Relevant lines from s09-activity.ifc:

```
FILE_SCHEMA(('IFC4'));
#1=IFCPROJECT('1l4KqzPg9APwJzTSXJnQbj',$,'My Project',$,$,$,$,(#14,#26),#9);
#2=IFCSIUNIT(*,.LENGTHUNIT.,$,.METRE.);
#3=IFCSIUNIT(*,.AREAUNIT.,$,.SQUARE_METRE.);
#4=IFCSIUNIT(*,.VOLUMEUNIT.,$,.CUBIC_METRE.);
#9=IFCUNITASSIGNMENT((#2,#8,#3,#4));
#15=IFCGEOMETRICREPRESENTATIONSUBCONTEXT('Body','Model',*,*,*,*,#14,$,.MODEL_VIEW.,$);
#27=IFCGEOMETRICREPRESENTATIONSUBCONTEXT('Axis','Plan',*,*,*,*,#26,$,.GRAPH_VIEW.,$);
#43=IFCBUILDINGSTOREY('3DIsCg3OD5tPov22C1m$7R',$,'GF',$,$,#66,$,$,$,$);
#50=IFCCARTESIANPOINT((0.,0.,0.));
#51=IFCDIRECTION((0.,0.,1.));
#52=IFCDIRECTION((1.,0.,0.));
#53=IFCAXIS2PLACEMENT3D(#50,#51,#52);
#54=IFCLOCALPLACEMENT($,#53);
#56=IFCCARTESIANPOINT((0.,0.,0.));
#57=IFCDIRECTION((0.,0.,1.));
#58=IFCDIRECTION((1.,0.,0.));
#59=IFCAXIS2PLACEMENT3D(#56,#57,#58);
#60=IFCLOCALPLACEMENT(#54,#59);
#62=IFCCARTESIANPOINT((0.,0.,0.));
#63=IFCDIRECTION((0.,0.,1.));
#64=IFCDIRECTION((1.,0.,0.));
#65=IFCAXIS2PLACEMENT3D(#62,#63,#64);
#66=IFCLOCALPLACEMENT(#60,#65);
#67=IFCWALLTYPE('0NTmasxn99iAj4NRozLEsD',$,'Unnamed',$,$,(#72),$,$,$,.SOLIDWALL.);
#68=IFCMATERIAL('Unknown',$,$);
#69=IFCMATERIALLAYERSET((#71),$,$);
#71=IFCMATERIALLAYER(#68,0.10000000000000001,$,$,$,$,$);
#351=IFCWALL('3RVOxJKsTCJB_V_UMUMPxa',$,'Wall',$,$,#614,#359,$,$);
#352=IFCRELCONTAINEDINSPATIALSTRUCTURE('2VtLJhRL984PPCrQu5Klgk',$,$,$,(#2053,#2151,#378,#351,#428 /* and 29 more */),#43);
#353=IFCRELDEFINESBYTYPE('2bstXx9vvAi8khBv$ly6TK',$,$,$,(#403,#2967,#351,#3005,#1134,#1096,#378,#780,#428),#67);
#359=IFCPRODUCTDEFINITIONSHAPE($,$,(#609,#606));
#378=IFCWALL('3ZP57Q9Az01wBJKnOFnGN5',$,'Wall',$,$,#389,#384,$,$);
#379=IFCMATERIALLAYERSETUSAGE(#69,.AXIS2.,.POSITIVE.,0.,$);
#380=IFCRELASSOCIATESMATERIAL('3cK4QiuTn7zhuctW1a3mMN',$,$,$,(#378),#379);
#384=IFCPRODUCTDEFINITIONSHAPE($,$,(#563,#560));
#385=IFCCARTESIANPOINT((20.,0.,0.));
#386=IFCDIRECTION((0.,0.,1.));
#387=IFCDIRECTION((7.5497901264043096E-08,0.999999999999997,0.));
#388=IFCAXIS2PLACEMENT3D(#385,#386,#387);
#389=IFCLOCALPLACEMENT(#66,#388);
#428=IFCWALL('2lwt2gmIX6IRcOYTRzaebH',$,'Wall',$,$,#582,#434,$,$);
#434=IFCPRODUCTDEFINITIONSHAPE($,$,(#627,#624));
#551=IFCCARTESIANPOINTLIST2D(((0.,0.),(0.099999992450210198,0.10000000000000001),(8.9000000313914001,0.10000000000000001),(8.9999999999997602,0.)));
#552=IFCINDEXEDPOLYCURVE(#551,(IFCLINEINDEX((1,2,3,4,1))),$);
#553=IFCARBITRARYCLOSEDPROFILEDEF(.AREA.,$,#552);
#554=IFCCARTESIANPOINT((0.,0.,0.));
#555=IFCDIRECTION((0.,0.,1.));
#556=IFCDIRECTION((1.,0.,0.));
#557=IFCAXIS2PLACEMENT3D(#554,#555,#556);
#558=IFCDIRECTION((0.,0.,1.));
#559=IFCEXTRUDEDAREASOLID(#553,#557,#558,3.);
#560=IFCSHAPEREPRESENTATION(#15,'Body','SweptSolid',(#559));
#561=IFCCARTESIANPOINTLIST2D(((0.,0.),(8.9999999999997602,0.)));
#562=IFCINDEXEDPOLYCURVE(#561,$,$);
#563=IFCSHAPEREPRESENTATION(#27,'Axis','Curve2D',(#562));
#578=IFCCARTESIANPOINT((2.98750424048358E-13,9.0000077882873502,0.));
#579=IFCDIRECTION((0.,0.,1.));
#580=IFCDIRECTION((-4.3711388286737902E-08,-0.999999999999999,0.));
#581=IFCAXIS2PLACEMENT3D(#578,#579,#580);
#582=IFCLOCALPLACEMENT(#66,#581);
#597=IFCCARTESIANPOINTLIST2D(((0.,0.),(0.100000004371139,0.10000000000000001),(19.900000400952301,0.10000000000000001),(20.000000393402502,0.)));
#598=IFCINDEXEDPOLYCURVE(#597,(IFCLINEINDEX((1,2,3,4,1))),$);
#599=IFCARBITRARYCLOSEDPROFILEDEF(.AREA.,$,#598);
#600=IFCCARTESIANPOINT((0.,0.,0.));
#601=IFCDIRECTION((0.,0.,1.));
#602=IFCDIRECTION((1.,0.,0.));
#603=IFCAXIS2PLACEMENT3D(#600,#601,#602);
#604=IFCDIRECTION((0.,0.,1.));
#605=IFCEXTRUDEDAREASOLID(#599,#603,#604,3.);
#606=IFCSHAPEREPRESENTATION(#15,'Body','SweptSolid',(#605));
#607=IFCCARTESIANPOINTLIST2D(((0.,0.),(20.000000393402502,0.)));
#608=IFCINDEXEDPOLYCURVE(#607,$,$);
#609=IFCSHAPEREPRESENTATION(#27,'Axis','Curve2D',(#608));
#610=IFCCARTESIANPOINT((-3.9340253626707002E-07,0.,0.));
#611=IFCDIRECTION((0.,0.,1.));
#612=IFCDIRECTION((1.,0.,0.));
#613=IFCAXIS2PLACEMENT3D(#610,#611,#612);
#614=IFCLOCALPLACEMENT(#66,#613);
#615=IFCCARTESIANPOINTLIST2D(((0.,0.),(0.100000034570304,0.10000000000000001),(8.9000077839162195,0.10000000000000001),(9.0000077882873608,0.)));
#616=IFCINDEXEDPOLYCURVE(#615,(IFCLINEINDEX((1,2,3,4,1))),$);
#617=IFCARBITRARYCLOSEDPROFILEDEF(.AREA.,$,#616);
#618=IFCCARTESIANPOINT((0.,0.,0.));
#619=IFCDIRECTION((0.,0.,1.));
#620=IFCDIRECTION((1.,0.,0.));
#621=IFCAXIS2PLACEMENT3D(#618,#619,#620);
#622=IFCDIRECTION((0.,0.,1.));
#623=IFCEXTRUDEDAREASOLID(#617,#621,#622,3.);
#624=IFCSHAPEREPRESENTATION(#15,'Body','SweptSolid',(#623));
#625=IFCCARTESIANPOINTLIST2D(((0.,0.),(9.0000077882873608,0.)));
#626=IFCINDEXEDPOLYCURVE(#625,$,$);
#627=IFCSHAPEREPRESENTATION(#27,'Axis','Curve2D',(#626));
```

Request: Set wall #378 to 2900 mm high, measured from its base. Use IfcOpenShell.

```python
import ifcopenshell
import ifcopenshell.geom
import ifcopenshell.util.representation
import ifcopenshell.util.shape

model = ifcopenshell.open("s09-activity.ifc")
settings = ifcopenshell.geom.settings()


def volume(element):
    """Net volume in cubic metres, openings subtracted."""
    shape = ifcopenshell.geom.create_shape(settings, element)
    return ifcopenshell.util.shape.get_volume(shape.geometry)


wall = model.by_id(378)
before = volume(wall)

body = ifcopenshell.util.representation.get_representation(wall, "Model", "Body")
solid = body.Items[0]
old_height = solid.Depth
solid.Depth = 2.9
after = volume(wall)

print(f"height {old_height:g} -> {solid.Depth:g}, volume {before:.3f} -> {after:.3f} m3")

model.write("s09-activity_v2.ifc")
```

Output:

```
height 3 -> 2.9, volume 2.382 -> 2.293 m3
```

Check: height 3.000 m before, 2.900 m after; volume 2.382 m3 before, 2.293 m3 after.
